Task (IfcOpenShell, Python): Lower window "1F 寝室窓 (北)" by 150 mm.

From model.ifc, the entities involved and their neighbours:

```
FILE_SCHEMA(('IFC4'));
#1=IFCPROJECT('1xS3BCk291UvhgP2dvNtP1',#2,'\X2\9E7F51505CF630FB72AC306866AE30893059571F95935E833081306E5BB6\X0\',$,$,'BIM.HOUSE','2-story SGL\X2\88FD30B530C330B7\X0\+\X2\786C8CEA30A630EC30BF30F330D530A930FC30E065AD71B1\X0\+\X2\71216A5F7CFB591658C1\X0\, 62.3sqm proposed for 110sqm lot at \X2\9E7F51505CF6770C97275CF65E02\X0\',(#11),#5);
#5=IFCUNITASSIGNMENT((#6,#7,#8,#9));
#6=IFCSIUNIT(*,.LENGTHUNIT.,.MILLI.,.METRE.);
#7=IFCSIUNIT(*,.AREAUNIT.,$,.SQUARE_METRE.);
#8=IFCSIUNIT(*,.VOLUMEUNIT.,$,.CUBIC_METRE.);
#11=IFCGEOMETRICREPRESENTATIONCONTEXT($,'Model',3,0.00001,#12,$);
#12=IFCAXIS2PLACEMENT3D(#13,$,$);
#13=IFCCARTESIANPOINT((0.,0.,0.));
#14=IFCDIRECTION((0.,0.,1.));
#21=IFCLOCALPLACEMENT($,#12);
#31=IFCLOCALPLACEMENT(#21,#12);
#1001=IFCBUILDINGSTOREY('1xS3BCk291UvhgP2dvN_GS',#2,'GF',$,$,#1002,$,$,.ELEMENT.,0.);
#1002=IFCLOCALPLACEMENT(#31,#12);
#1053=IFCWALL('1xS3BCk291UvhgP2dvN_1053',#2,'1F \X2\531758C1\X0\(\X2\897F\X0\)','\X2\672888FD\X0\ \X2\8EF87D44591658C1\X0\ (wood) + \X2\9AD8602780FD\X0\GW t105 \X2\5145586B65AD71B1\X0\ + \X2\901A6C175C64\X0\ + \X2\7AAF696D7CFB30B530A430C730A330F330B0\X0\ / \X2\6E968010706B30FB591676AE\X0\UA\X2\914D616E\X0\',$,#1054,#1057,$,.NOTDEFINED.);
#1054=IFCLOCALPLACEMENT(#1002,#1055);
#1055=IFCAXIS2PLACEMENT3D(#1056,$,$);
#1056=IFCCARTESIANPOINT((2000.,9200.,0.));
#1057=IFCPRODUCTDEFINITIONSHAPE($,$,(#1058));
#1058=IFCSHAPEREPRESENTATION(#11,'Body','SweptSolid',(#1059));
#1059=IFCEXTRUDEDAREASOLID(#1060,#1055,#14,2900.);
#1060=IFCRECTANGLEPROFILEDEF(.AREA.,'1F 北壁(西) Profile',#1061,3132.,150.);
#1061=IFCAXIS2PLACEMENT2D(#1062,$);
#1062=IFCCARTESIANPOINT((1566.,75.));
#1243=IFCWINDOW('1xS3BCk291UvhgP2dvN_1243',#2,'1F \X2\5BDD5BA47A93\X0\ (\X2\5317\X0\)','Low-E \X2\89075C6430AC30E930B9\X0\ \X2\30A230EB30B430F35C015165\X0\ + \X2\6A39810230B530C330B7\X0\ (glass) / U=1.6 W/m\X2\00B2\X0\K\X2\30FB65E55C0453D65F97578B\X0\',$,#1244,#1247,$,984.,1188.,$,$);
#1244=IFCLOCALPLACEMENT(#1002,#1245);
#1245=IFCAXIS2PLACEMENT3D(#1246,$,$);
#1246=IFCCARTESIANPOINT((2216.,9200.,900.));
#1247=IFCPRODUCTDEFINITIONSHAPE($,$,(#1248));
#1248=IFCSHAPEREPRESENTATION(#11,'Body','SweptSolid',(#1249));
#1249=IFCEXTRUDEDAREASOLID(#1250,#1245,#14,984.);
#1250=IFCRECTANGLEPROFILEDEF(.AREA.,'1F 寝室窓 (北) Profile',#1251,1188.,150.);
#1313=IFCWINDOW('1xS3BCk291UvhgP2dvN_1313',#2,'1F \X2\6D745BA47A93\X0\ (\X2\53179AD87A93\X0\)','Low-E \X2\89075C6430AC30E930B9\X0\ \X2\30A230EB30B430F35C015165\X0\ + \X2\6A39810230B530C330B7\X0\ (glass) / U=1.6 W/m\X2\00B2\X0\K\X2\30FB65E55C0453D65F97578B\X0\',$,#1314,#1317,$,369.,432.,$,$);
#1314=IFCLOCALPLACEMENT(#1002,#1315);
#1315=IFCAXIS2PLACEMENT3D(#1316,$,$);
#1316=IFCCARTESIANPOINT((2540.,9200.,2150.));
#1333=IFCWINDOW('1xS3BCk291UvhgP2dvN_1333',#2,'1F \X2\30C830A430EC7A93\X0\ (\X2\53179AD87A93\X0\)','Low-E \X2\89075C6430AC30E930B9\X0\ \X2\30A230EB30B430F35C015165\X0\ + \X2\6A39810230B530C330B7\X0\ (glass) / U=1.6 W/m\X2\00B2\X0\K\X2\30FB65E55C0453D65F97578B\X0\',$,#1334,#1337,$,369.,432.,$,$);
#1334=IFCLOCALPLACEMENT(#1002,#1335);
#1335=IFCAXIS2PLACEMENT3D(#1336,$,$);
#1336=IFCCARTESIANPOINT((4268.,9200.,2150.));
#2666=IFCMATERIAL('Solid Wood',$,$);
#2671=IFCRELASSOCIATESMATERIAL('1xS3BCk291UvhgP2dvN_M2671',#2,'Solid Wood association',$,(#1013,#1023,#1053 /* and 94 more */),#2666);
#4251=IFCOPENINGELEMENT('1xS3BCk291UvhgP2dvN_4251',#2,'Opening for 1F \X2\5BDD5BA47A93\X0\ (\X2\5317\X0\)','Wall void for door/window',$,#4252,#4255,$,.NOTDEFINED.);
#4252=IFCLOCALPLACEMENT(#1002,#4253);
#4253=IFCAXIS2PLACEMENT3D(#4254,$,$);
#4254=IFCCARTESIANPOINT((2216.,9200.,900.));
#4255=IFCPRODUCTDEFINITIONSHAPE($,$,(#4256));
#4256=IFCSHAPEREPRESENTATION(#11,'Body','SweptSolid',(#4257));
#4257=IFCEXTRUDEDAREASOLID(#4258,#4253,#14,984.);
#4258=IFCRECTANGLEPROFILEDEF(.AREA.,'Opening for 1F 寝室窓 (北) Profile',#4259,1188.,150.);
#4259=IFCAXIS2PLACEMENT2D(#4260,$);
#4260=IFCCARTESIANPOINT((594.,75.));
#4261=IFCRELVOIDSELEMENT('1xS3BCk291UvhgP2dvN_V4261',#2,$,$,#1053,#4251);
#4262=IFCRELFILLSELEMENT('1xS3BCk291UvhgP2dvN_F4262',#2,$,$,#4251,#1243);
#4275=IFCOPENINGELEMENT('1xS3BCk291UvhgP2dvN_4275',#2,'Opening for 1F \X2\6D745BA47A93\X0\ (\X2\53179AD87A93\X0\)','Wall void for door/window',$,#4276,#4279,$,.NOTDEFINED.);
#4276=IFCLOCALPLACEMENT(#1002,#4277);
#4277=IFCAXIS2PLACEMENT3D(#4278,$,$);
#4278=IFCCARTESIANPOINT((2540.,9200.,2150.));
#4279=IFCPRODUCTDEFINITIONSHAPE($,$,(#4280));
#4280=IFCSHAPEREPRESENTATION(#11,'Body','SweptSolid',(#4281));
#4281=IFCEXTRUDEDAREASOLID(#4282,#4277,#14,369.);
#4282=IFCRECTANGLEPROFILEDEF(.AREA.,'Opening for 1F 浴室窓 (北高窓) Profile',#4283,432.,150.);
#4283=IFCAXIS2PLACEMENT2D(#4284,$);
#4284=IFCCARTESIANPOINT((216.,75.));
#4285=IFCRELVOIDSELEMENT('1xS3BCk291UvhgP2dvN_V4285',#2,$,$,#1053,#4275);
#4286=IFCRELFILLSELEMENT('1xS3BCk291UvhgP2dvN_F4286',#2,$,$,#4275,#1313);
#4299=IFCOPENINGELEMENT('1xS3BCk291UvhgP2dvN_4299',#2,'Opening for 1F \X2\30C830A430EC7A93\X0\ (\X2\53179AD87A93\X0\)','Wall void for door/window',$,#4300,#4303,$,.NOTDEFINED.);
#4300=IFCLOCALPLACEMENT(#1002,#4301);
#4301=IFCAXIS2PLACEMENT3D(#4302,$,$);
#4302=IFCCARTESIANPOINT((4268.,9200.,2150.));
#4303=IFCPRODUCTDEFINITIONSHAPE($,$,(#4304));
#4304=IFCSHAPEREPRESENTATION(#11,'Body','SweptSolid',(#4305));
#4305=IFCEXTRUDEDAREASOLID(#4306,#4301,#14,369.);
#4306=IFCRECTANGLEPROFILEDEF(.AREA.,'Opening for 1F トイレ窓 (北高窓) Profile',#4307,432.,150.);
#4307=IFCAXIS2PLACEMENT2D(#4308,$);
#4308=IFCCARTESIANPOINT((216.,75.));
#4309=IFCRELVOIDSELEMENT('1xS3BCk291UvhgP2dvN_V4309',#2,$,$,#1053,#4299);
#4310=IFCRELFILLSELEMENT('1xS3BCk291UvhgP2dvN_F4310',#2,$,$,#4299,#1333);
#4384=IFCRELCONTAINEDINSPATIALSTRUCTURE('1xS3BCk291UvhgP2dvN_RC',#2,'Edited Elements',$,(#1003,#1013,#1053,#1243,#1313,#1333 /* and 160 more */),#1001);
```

```python
import numpy as np
import ifcopenshell
import ifcopenshell.api.geometry
import ifcopenshell.util.placement
import ifcopenshell.util.unit

model = ifcopenshell.open("model.ifc")
unit_scale = ifcopenshell.util.unit.calculate_unit_scale(model)

window = model.by_guid("1xS3BCk291UvhgP2dvN_1243")
opening = window.FillsVoids[0].RelatingOpeningElement
dz = -150.0

shift = np.array([0.0, 0.0, dz])
# The window is not placed relative to its opening, so move both.
for product in (opening, window):
    matrix = ifcopenshell.util.placement.get_local_placement(product.ObjectPlacement)
    matrix[:3, 3] += shift
    ifcopenshell.api.geometry.edit_object_placement(model, product=product, matrix=matrix, is_si=False)

print(f"moved by {dz * unit_scale:+.3f} m")

model.write("model_edited.ifc")
```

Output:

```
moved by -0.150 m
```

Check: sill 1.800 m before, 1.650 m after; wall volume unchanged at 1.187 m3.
